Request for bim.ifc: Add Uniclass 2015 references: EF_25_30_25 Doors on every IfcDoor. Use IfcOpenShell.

First a look at what the model holds.

```python
import ifcopenshell

model = ifcopenshell.open("bim.ifc")
print(model.schema)
print("classifications:", [c.Name for c in model.by_type("IfcClassification")])
for ifc_class in ("IfcDoor", "IfcRoof", "IfcStair", "IfcWall", "IfcWindow"):
    print(ifc_class, len(model.by_type(ifc_class)))
```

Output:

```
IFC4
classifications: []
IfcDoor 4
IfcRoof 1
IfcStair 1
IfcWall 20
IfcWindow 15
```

```python
import ifcopenshell
import ifcopenshell.api.classification

model = ifcopenshell.open("bim.ifc")

system = ifcopenshell.api.classification.add_classification(model, classification="Uniclass 2015")

codes = {
    "IfcDoor": ("EF_25_30_25", "Doors"),
}
for ifc_class, (code, name) in codes.items():
    products = model.by_type(ifc_class)
    ifcopenshell.api.classification.add_reference(
        model, products=products, classification=system, identification=code, name=name
    )
    print(code, len(products))

model.write("bim_updated.ifc")
```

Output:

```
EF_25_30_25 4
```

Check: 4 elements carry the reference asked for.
